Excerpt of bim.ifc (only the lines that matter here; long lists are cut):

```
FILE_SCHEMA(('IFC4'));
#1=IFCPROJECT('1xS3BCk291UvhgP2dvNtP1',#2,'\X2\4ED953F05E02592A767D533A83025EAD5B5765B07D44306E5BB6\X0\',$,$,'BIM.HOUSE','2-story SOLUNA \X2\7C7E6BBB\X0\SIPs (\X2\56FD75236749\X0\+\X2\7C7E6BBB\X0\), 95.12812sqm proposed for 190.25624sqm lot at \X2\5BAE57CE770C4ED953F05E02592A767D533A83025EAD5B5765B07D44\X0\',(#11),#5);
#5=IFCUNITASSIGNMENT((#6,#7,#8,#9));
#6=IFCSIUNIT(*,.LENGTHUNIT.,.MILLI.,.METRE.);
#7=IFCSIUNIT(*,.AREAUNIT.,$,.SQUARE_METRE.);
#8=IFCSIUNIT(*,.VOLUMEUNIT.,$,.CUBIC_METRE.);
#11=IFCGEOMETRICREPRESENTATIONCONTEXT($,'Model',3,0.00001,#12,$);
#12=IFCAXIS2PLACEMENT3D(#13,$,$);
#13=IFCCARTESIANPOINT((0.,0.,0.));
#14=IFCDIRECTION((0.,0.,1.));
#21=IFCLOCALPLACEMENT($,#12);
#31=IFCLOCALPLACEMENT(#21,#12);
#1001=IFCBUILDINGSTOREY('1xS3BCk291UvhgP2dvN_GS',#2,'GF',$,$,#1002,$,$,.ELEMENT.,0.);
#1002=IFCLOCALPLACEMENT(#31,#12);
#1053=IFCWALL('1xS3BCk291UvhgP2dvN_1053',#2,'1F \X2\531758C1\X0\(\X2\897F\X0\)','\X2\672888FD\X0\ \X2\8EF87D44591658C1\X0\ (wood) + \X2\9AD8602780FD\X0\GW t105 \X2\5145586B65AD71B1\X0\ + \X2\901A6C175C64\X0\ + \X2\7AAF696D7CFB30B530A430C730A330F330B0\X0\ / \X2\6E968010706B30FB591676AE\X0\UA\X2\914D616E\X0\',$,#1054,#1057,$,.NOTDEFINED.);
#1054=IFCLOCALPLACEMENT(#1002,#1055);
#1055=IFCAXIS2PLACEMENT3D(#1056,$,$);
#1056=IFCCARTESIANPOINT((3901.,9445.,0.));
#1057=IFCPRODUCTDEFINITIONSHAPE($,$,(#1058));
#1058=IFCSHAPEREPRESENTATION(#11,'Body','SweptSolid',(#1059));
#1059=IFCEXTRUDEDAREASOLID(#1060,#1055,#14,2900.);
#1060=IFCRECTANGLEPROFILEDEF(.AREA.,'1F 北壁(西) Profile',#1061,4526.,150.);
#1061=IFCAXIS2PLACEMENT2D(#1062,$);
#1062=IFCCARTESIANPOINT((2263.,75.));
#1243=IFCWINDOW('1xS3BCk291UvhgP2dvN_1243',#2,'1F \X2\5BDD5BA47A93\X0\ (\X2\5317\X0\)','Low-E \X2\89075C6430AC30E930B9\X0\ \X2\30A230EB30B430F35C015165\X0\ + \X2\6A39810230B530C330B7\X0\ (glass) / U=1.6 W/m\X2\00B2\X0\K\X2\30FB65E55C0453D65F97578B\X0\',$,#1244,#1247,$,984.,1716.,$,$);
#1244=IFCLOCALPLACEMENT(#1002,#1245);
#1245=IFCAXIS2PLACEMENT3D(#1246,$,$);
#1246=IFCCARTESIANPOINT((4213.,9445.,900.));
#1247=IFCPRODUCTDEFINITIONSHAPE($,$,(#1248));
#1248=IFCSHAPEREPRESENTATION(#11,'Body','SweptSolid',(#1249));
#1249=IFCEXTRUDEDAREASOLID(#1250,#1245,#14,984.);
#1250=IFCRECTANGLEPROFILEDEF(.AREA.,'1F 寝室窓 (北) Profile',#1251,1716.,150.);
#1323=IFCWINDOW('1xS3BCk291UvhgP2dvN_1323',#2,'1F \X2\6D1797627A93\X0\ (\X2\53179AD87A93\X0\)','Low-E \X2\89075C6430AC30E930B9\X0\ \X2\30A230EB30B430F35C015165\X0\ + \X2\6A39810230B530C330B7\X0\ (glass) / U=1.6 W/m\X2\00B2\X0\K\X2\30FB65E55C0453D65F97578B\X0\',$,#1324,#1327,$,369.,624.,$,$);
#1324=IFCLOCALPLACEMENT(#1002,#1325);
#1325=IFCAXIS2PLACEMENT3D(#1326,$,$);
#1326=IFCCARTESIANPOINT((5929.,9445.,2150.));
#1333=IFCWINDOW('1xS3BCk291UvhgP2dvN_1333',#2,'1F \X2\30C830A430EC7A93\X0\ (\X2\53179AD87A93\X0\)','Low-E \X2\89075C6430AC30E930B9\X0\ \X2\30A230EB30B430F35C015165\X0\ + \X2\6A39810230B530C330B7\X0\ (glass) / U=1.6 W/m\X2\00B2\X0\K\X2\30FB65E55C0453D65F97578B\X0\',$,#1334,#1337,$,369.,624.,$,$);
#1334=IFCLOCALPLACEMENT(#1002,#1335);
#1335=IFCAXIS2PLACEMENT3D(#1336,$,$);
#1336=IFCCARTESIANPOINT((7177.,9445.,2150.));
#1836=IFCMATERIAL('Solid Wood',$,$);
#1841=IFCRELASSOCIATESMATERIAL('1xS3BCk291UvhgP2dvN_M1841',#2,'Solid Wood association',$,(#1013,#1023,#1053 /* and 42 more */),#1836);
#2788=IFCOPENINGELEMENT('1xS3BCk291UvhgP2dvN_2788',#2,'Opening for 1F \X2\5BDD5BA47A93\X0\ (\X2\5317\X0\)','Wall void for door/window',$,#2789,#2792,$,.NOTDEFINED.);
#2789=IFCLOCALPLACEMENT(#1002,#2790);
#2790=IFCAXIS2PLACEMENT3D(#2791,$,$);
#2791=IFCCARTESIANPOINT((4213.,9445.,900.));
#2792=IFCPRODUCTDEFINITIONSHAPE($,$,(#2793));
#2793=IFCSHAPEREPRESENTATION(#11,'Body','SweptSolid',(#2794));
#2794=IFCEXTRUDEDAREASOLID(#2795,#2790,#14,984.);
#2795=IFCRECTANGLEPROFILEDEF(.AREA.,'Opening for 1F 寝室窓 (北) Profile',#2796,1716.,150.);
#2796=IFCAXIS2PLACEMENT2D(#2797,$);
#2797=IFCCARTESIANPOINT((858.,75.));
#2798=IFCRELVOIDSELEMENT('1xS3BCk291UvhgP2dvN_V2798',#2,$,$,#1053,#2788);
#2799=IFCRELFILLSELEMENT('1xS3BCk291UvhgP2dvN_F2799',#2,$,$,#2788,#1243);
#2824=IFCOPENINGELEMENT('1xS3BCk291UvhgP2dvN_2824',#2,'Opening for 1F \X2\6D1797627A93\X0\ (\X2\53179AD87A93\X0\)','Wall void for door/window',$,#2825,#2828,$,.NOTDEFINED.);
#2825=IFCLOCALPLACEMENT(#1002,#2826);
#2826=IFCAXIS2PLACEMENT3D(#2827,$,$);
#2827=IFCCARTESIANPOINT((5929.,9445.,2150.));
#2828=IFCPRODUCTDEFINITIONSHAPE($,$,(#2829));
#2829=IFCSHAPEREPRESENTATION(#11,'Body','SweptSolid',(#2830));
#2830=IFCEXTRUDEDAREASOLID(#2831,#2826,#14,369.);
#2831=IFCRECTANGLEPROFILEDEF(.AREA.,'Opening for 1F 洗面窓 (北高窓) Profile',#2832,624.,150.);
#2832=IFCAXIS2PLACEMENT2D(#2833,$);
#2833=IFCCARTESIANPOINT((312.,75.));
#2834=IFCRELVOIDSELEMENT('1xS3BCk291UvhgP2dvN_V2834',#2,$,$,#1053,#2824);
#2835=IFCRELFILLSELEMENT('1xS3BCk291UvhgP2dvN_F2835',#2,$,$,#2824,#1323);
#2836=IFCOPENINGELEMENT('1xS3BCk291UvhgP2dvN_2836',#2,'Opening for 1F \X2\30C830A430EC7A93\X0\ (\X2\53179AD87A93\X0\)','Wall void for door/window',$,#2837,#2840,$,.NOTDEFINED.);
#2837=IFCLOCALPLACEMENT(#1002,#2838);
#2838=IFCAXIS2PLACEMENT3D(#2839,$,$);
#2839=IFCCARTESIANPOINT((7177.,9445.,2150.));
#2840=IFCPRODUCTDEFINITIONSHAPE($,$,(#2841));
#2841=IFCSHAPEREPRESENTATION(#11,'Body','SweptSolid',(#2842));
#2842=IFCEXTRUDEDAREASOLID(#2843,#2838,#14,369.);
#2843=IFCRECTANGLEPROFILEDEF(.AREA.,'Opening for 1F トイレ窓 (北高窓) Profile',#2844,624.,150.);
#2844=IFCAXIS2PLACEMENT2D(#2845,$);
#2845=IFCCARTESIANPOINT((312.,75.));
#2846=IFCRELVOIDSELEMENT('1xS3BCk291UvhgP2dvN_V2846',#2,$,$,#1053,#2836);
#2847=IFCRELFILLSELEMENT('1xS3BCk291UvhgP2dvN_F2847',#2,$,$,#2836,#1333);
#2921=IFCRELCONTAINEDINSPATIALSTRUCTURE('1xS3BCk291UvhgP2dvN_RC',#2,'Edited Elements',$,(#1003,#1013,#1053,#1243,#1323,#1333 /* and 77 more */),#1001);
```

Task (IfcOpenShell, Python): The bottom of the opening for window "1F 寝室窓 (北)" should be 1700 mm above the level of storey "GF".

```python
import numpy as np
import ifcopenshell
import ifcopenshell.api.geometry
import ifcopenshell.geom
import ifcopenshell.util.element
import ifcopenshell.util.placement
import ifcopenshell.util.shape
import ifcopenshell.util.unit

model = ifcopenshell.open("bim.ifc")
unit_scale = ifcopenshell.util.unit.calculate_unit_scale(model)

window = model.by_guid("1xS3BCk291UvhgP2dvN_1243")
opening = window.FillsVoids[0].RelatingOpeningElement
storey = ifcopenshell.util.element.get_container(window, ifc_class="IfcBuildingStorey")
level = ifcopenshell.util.placement.get_local_placement(storey.ObjectPlacement)[2, 3]

# The opening's origin need not be at the sill, so measure its lowest point.
shape = ifcopenshell.geom.create_shape(ifcopenshell.geom.settings(), opening)
bottom = ifcopenshell.util.shape.get_shape_bottom_elevation(shape, shape.geometry) / unit_scale
dz = level + 1.7 / unit_scale - bottom

shift = np.array([0.0, 0.0, dz])
# The window is not placed relative to its opening, so move both.
for product in (opening, window):
    matrix = ifcopenshell.util.placement.get_local_placement(product.ObjectPlacement)
    matrix[:3, 3] += shift
    ifcopenshell.api.geometry.edit_object_placement(model, product=product, matrix=matrix, is_si=False)

print(f"moved by {dz * unit_scale:+.3f} m")

model.write("bim_edited.ifc")
```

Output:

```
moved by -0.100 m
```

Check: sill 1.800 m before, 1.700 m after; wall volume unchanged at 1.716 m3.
